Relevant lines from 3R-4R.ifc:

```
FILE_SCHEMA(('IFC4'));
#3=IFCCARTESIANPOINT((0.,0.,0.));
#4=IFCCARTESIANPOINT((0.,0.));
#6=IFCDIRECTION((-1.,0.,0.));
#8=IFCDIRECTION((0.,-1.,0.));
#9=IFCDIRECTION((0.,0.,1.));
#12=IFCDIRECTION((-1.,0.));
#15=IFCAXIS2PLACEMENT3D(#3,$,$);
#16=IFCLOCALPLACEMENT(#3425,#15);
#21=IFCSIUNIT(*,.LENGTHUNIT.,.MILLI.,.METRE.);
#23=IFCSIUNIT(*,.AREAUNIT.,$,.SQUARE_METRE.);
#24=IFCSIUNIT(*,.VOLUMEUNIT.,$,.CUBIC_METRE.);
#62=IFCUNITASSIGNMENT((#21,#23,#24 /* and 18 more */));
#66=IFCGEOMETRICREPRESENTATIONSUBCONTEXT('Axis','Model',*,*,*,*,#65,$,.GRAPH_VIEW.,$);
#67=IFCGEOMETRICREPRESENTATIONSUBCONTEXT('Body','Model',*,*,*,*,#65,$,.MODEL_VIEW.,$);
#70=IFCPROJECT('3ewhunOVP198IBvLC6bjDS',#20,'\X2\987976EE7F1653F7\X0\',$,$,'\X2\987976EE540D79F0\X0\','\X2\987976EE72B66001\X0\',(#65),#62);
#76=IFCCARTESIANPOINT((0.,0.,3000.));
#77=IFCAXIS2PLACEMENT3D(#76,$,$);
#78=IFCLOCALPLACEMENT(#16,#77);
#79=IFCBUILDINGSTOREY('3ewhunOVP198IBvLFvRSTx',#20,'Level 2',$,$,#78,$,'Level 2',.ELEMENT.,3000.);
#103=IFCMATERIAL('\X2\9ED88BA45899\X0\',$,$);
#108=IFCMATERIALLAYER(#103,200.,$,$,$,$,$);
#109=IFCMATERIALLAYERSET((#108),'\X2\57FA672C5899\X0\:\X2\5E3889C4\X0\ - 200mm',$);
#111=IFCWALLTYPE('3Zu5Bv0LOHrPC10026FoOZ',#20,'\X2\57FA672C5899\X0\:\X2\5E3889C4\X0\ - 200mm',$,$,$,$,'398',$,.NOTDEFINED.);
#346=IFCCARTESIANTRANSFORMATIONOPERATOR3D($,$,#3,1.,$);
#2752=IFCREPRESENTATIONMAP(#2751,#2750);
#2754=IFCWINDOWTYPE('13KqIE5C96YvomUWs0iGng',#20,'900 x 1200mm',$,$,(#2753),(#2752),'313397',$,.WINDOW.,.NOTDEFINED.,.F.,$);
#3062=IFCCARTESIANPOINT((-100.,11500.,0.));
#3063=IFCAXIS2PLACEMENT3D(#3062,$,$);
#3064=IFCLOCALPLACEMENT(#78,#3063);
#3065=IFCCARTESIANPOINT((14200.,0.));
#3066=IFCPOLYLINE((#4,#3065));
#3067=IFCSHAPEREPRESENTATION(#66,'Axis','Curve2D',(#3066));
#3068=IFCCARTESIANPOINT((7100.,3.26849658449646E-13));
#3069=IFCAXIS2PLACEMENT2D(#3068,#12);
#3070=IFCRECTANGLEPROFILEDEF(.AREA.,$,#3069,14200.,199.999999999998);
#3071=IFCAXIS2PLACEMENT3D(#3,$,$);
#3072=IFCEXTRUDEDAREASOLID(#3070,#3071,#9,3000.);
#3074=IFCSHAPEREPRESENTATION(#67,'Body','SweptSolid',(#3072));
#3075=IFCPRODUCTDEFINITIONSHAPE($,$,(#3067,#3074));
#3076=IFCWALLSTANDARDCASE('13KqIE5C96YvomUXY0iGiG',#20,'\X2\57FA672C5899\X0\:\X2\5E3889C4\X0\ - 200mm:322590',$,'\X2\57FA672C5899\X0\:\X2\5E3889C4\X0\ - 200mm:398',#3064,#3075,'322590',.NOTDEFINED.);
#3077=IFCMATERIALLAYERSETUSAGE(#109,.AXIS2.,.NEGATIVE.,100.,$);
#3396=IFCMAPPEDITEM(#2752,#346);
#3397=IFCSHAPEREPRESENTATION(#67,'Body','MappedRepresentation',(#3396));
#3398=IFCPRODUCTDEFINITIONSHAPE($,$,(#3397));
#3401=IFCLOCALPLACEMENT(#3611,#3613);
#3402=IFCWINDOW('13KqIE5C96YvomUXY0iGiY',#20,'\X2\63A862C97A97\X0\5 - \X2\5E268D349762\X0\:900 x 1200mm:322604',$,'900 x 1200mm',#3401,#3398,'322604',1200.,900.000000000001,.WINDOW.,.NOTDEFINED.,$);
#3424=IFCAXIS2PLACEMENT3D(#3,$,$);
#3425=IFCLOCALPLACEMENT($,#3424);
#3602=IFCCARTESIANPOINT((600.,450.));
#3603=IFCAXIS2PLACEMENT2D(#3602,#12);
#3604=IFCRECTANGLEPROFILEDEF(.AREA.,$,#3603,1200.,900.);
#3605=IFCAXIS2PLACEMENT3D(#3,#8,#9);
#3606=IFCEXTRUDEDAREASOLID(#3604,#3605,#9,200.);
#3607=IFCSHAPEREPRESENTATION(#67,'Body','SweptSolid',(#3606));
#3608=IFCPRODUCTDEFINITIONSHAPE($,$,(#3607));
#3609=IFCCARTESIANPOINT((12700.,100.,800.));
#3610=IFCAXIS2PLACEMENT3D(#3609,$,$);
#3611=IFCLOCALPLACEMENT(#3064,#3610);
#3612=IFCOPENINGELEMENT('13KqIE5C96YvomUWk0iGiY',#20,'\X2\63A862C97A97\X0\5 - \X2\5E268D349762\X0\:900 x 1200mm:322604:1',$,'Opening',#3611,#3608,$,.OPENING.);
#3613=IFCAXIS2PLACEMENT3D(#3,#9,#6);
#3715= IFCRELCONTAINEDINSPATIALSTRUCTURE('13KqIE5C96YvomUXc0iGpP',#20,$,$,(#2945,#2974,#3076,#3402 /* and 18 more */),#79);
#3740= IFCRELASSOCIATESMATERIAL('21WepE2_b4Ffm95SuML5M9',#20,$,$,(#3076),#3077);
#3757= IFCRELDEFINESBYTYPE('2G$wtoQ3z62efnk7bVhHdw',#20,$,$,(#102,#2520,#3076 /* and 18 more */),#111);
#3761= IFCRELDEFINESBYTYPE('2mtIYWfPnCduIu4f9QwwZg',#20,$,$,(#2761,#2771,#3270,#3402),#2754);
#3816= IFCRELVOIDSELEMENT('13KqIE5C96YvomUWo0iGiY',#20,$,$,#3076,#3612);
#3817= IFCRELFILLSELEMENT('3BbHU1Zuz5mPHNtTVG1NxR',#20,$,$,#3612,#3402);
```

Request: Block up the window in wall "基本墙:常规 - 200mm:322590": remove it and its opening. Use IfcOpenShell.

```python
import ifcopenshell
import ifcopenshell.api.feature
import ifcopenshell.api.root
import ifcopenshell.geom
import ifcopenshell.util.shape

model = ifcopenshell.open("3R-4R.ifc")
settings = ifcopenshell.geom.settings()


def volume(element):
    """Net volume in cubic metres, openings subtracted."""
    shape = ifcopenshell.geom.create_shape(settings, element)
    return ifcopenshell.util.shape.get_volume(shape.geometry)


window = model.by_guid("13KqIE5C96YvomUXY0iGiY")
opening = window.FillsVoids[0].RelatingOpeningElement
wall = opening.VoidsElements[0].RelatingBuildingElement
before = volume(wall)

ifcopenshell.api.root.remove_product(model, product=window)
ifcopenshell.api.feature.remove_feature(model, feature=opening)

after = volume(wall)

print(f"wall volume {before:.3f} -> {after:.3f} m3")

model.write("3R-4R-out.ifc")
```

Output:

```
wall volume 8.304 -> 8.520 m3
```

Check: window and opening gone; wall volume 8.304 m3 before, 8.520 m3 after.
